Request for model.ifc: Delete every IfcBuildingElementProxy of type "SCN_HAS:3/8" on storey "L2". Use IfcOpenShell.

First a look at what the model holds.

```python
import ifcopenshell
import ifcopenshell.util.element

model = ifcopenshell.open("model.ifc")
print(model.schema)
storey = next(s for s in model.by_type("IfcBuildingStorey") if s.Name == "L2")
proxies = [e for e in ifcopenshell.util.element.get_decomposition(storey) if e.is_a("IfcBuildingElementProxy")]
seen = {}
for e in proxies:
    element_type = ifcopenshell.util.element.get_type(e)
    name = element_type.Name if element_type not in (None, e) else None
    seen[name] = seen.get(name, 0) + 1
for name, count in sorted(seen.items(), key=str):
    print(count, "x", name)
```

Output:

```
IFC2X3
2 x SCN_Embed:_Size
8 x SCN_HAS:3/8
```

```python
import ifcopenshell
import ifcopenshell.api.root
import ifcopenshell.util.element

model = ifcopenshell.open("model.ifc")

storey = next(s for s in model.by_type("IfcBuildingStorey") if s.Name == "L2")
proxies = [e for e in ifcopenshell.util.element.get_decomposition(storey) if e.is_a("IfcBuildingElementProxy")]
targets = [e for e in proxies if (t := ifcopenshell.util.element.get_type(e)) not in (None, e) and t.Name == "SCN_HAS:3/8"]

for e in targets:
    ifcopenshell.api.root.remove_product(model, product=e)
print(len(targets), "removed")

model.write("model_v2.ifc")
```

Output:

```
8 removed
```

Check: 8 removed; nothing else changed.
